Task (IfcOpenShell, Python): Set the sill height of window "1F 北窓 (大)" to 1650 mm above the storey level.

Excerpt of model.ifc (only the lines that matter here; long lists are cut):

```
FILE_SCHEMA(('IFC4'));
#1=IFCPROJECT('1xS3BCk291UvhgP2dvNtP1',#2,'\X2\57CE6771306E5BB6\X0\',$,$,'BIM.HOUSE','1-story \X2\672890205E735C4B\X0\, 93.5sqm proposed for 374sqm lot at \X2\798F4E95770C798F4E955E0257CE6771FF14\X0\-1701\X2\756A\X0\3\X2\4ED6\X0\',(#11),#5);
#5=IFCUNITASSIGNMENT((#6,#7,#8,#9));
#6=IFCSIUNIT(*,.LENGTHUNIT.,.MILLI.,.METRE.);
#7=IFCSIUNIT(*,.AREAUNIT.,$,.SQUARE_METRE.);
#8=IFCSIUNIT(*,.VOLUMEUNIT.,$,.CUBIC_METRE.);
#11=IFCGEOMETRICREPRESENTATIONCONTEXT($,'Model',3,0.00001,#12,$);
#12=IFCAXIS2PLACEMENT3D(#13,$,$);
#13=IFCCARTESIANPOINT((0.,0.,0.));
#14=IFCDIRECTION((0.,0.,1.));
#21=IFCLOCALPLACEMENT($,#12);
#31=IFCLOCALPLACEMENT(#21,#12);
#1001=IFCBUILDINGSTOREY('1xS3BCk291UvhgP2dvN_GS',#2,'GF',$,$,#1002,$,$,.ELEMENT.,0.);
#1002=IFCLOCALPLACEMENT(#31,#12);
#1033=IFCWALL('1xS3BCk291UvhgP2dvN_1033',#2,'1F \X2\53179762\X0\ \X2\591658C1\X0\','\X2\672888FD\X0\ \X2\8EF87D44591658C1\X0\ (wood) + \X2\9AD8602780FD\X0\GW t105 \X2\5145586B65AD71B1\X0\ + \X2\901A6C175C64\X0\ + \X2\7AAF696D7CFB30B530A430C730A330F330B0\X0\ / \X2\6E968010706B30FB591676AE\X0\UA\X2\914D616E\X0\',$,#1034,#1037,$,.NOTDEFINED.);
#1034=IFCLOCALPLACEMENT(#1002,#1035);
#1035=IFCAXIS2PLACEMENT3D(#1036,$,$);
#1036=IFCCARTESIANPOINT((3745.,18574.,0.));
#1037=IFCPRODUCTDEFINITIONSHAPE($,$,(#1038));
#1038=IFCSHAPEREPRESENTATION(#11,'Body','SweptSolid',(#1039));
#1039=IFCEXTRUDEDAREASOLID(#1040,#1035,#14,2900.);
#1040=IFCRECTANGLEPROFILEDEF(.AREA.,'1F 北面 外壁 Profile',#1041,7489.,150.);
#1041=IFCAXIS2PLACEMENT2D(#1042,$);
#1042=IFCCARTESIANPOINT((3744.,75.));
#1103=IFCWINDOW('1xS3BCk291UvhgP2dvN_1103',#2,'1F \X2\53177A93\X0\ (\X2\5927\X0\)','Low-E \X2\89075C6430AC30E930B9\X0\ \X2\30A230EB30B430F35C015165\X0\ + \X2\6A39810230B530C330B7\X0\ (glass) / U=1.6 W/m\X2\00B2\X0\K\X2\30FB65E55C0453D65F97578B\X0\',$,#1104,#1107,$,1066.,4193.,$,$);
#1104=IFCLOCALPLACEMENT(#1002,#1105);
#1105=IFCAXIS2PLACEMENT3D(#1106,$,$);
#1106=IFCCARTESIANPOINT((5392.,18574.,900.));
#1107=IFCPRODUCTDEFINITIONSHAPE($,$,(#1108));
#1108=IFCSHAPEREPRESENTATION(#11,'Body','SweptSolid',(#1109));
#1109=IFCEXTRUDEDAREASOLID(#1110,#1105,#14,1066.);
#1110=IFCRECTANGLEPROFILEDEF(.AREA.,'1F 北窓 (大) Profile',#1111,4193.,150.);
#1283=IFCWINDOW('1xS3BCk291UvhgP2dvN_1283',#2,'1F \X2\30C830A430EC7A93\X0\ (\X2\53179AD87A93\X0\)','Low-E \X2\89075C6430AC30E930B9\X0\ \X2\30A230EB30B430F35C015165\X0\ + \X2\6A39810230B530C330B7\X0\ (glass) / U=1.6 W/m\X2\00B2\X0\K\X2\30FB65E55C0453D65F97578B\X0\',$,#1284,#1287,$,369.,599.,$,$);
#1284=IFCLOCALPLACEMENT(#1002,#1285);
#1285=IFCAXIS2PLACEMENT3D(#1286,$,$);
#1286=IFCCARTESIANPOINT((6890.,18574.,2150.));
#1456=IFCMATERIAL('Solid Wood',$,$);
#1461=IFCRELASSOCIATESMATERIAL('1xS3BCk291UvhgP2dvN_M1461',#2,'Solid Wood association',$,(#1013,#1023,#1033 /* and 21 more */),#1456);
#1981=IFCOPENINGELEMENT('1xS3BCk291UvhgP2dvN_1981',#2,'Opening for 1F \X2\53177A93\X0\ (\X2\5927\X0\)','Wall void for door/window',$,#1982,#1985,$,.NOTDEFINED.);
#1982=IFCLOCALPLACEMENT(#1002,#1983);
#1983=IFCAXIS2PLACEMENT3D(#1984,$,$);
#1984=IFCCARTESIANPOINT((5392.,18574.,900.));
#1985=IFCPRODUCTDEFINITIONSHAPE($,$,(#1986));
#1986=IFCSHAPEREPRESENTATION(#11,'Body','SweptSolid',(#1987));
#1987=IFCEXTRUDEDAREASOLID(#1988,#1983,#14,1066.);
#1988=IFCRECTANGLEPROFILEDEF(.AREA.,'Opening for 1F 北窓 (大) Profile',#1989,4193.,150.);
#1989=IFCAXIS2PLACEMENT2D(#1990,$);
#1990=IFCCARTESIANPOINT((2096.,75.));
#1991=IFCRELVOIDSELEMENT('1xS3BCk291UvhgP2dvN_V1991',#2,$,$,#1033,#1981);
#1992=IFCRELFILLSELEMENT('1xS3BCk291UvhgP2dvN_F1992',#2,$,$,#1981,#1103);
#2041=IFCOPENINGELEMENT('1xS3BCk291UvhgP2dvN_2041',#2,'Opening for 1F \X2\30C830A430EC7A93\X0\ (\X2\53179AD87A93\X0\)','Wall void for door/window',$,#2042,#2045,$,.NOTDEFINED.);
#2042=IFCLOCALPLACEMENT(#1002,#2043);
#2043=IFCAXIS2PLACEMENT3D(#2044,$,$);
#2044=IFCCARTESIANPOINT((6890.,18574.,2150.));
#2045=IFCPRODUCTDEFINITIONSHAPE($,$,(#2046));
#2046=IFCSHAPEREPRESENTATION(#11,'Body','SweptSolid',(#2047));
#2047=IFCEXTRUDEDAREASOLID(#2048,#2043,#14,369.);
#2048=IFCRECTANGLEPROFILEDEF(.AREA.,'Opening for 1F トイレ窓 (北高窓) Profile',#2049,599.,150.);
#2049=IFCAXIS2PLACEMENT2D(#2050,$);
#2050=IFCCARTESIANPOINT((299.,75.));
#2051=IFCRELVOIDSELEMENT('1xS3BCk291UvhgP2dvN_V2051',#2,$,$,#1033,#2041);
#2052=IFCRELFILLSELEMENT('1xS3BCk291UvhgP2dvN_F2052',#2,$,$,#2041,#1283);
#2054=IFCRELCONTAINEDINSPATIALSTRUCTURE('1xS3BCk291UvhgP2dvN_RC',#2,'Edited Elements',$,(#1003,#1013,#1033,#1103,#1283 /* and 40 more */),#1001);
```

```python
import numpy as np
import ifcopenshell
import ifcopenshell.api.geometry
import ifcopenshell.geom
import ifcopenshell.util.element
import ifcopenshell.util.placement
import ifcopenshell.util.shape
import ifcopenshell.util.unit

model = ifcopenshell.open("model.ifc")
unit_scale = ifcopenshell.util.unit.calculate_unit_scale(model)

window = model.by_guid("1xS3BCk291UvhgP2dvN_1103")
opening = window.FillsVoids[0].RelatingOpeningElement
storey = ifcopenshell.util.element.get_container(window, ifc_class="IfcBuildingStorey")
level = ifcopenshell.util.placement.get_local_placement(storey.ObjectPlacement)[2, 3]

# The opening's origin need not be at the sill, so measure its lowest point.
shape = ifcopenshell.geom.create_shape(ifcopenshell.geom.settings(), opening)
bottom = ifcopenshell.util.shape.get_shape_bottom_elevation(shape, shape.geometry) / unit_scale
dz = level + 1.65 / unit_scale - bottom

shift = np.array([0.0, 0.0, dz])
# The window is not placed relative to its opening, so move both.
for product in (opening, window):
    matrix = ifcopenshell.util.placement.get_local_placement(product.ObjectPlacement)
    matrix[:3, 3] += shift
    ifcopenshell.api.geometry.edit_object_placement(model, product=product, matrix=matrix, is_si=False)

print(f"moved by {dz * unit_scale:+.3f} m")

model.write("model_edited.ifc")
```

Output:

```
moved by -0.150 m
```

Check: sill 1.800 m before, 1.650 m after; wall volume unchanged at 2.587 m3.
